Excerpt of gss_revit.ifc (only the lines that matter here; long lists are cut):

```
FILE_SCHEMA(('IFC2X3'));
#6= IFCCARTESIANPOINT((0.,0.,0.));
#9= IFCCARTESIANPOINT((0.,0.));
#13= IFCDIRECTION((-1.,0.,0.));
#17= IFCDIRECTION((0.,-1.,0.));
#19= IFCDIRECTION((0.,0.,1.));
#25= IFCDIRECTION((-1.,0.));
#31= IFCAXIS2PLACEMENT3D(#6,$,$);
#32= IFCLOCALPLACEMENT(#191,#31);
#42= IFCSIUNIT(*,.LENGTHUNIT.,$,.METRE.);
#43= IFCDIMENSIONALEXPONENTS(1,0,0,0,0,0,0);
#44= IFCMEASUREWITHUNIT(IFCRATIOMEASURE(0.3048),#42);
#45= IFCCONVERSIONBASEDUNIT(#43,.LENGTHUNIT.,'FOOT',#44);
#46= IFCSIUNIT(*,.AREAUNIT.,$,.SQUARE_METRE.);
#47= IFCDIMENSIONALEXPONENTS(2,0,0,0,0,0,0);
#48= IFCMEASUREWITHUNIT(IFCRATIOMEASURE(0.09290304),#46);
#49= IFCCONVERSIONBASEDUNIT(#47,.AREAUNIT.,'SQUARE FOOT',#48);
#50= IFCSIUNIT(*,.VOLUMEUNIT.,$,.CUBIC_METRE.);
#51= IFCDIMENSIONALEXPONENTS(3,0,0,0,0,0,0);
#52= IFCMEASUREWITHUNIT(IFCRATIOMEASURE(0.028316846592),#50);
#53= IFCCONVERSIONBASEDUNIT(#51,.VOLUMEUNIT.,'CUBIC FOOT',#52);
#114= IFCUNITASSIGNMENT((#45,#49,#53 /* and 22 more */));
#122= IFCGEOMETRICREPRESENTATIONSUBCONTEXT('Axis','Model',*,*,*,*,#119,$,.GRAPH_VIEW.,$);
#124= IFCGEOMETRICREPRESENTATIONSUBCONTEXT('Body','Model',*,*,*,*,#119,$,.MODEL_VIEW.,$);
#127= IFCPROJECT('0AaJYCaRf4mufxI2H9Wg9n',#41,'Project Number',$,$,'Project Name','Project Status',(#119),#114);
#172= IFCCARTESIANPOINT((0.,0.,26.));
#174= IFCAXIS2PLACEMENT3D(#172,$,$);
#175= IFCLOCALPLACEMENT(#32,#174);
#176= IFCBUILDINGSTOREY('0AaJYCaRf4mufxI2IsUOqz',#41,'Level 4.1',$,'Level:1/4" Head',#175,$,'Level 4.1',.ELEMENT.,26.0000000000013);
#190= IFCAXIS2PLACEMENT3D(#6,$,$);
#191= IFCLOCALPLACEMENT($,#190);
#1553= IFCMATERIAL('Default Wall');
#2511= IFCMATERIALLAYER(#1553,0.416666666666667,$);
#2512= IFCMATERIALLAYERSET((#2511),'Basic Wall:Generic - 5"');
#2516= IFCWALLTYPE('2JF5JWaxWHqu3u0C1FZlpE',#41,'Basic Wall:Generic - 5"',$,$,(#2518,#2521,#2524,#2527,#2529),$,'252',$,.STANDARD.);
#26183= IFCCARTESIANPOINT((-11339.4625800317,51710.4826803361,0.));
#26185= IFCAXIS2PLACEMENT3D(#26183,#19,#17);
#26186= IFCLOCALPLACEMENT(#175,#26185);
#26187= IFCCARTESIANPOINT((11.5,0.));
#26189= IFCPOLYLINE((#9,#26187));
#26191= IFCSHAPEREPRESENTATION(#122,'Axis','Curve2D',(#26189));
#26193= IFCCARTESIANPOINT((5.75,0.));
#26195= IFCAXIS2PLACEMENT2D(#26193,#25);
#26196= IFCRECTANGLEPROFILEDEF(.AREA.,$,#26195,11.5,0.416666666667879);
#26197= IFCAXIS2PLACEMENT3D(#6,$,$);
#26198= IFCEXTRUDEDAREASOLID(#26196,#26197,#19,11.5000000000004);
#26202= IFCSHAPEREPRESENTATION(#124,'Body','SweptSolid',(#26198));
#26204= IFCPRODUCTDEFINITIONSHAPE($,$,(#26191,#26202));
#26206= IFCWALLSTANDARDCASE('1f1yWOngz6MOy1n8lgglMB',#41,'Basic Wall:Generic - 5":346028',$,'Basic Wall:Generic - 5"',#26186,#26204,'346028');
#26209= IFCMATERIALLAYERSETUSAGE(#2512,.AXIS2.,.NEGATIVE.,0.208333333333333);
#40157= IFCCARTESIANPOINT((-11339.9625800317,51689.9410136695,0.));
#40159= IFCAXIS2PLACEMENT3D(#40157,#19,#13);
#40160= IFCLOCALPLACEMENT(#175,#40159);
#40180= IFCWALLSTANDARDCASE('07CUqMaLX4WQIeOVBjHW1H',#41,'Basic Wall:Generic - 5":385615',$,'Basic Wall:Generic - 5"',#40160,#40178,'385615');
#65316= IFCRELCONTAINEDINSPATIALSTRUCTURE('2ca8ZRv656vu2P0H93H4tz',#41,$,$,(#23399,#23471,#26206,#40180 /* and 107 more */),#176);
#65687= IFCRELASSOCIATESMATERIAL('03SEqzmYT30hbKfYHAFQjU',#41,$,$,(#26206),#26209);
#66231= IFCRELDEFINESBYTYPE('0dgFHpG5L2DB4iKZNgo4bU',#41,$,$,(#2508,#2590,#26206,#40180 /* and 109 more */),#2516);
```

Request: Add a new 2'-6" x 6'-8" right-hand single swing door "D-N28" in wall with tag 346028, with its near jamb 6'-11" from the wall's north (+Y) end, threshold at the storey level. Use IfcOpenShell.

```python
import numpy as np
import ifcopenshell
import ifcopenshell.api.feature
import ifcopenshell.api.geometry
import ifcopenshell.api.root
import ifcopenshell.api.spatial
import ifcopenshell.api.type
import ifcopenshell.geom
import ifcopenshell.util.element
import ifcopenshell.util.placement
import ifcopenshell.util.representation
import ifcopenshell.util.shape
import ifcopenshell.util.unit

model = ifcopenshell.open("gss_revit.ifc")
unit_scale = ifcopenshell.util.unit.calculate_unit_scale(model)
settings = ifcopenshell.geom.settings()


def volume(element):
    """Net volume in cubic metres, openings subtracted."""
    shape = ifcopenshell.geom.create_shape(settings, element)
    return ifcopenshell.util.shape.get_volume(shape.geometry)


wall = model.by_id(26206)
storey = ifcopenshell.util.element.get_container(wall, ifc_class="IfcBuildingStorey")
context = ifcopenshell.util.representation.get_context(model, "Model", "Body", "MODEL_VIEW")
before = volume(wall)

width, height, from_end, sill = 0.762, 2.032, 2.1082, 0.0  # metres

# The wall runs along its own X axis, and the end named is its -X end.
wall_shape = ifcopenshell.geom.create_shape(settings, wall)
x, y, z = ifcopenshell.util.shape.get_vertices(wall_shape.geometry).T
start = x.min() + from_end
face, thickness = float(y.min()), float(y.max() - y.min())
wall_matrix = ifcopenshell.util.placement.get_local_placement(wall.ObjectPlacement)
level = ifcopenshell.util.placement.get_local_placement(storey.ObjectPlacement)[2, 3]


def in_wall(x, y):
    """Placement at x, y metres in the wall's axes, at sill height."""
    matrix = wall_matrix.copy()
    matrix[:, 3] = wall_matrix @ np.array([x / unit_scale, y / unit_scale, 0.0, 1.0])
    matrix[2, 3] = level + sill / unit_scale
    return matrix


# Opening: a box that overshoots both wall faces by 50 mm.
opening = ifcopenshell.api.root.create_entity(model, ifc_class="IfcOpeningElement")
box = ifcopenshell.api.geometry.add_wall_representation(
    model, context=context, length=width, height=height, thickness=thickness + 0.1
)
ifcopenshell.api.geometry.assign_representation(model, product=opening, representation=box)
ifcopenshell.api.geometry.edit_object_placement(model, product=opening, matrix=in_wall(start, face - 0.05), is_si=False)
ifcopenshell.api.feature.add_feature(model, feature=opening, element=wall)

door = ifcopenshell.api.root.create_entity(model, ifc_class="IfcDoor", name="D-N28")
door.OverallWidth, door.OverallHeight = width / unit_scale, height / unit_scale
body = ifcopenshell.api.geometry.add_door_representation(
    model,
    context=context,
    overall_width=door.OverallWidth,
    overall_height=door.OverallHeight,
    operation_type="SINGLE_SWING_RIGHT",
    lining_properties={"LiningDepth": thickness / unit_scale, "ThresholdDepth": thickness / unit_scale},
)
ifcopenshell.api.geometry.assign_representation(model, product=door, representation=body)
ifcopenshell.api.spatial.assign_container(model, products=[door], relating_structure=storey)
fills = ifcopenshell.api.feature.add_filling(model, opening=opening, element=door)
fills.OwnerHistory = door.OwnerHistory  # required in IFC2X3

# IFC2X3 keeps the operation on the door style.
style = ifcopenshell.api.root.create_entity(model, ifc_class="IfcDoorStyle", name="D-N28")
style.OperationType, style.ConstructionType = "SINGLE_SWING_RIGHT", "NOTDEFINED"
style.ParameterTakesPrecedence = style.Sizeable = False
ifcopenshell.api.type.assign_type(model, related_objects=[door], relating_type=style)

# The lining spans the wall, so the door starts at the wall face.
ifcopenshell.api.geometry.edit_object_placement(model, product=door, matrix=in_wall(start, face), is_si=False)

after = volume(wall)

print(f"wall volume {before:.3f} -> {after:.3f} m3")

model.write("gss_revit_v2.ifc")
```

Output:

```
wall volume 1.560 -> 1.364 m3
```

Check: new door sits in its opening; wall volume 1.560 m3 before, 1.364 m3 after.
